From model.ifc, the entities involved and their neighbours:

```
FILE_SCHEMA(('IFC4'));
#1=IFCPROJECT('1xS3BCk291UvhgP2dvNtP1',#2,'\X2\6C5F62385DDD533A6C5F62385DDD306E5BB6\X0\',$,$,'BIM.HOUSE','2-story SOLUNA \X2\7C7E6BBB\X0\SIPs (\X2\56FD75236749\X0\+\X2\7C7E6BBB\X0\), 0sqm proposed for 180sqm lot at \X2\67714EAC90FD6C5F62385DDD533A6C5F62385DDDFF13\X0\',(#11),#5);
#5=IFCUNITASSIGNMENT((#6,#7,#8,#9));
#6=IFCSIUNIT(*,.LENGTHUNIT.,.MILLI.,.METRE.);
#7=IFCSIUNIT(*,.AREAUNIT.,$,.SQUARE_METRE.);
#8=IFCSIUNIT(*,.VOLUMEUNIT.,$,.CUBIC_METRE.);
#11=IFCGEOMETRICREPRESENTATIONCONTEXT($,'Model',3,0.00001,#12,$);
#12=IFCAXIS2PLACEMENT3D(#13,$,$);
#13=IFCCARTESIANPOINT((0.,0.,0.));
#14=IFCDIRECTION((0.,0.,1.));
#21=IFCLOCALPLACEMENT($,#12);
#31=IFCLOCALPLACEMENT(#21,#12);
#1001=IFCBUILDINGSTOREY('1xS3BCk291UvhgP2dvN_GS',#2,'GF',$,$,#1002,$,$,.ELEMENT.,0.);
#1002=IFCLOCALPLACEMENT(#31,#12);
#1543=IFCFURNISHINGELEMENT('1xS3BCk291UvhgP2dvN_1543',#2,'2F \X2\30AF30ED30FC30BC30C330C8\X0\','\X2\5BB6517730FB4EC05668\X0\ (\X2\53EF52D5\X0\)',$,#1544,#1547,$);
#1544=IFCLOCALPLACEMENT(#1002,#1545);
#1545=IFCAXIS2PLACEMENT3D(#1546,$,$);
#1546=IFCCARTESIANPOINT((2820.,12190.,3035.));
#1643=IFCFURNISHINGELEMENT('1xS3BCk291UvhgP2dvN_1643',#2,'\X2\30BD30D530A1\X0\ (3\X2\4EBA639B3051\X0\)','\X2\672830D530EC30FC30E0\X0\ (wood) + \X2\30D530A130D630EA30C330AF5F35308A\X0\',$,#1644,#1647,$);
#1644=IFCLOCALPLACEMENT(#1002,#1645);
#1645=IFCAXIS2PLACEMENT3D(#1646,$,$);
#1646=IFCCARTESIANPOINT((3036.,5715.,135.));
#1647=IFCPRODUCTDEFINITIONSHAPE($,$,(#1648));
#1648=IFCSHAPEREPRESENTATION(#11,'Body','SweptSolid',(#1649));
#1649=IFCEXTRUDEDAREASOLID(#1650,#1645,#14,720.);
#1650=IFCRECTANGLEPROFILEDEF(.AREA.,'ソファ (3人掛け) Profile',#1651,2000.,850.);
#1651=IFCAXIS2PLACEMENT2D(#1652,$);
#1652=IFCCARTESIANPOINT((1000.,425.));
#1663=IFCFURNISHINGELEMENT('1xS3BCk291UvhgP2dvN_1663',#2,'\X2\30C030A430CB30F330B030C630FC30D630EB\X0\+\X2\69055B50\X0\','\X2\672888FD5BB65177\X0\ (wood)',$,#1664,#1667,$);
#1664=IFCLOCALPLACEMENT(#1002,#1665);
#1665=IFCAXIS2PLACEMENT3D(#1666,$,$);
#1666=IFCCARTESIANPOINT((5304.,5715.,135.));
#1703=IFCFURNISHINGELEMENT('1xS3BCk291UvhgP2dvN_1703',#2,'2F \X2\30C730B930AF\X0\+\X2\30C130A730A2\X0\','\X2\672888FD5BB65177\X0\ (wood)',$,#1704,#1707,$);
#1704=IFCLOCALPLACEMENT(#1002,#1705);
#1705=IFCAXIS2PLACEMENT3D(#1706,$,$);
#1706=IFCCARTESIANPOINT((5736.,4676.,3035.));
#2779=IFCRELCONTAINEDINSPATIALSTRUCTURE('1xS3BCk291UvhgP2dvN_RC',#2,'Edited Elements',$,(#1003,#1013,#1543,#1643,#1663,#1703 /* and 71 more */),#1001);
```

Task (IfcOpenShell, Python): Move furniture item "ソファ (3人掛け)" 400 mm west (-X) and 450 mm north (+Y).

```python
import ifcopenshell
import ifcopenshell.api.geometry
import ifcopenshell.util.placement

model = ifcopenshell.open("model.ifc")

item = model.by_guid("1xS3BCk291UvhgP2dvN_1643")
matrix = ifcopenshell.util.placement.get_local_placement(item.ObjectPlacement)
matrix[0, 3] -= 400.0
matrix[1, 3] += 450.0
ifcopenshell.api.geometry.edit_object_placement(model, product=item, matrix=matrix, is_si=False)

print(ifcopenshell.util.placement.get_local_placement(item.ObjectPlacement).round(3) + 0.0)

model.write("model_updated.ifc")
```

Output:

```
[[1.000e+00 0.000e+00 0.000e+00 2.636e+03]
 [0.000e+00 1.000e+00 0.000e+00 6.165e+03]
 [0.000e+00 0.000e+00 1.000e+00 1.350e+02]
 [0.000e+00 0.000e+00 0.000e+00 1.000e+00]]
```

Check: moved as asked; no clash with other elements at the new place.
